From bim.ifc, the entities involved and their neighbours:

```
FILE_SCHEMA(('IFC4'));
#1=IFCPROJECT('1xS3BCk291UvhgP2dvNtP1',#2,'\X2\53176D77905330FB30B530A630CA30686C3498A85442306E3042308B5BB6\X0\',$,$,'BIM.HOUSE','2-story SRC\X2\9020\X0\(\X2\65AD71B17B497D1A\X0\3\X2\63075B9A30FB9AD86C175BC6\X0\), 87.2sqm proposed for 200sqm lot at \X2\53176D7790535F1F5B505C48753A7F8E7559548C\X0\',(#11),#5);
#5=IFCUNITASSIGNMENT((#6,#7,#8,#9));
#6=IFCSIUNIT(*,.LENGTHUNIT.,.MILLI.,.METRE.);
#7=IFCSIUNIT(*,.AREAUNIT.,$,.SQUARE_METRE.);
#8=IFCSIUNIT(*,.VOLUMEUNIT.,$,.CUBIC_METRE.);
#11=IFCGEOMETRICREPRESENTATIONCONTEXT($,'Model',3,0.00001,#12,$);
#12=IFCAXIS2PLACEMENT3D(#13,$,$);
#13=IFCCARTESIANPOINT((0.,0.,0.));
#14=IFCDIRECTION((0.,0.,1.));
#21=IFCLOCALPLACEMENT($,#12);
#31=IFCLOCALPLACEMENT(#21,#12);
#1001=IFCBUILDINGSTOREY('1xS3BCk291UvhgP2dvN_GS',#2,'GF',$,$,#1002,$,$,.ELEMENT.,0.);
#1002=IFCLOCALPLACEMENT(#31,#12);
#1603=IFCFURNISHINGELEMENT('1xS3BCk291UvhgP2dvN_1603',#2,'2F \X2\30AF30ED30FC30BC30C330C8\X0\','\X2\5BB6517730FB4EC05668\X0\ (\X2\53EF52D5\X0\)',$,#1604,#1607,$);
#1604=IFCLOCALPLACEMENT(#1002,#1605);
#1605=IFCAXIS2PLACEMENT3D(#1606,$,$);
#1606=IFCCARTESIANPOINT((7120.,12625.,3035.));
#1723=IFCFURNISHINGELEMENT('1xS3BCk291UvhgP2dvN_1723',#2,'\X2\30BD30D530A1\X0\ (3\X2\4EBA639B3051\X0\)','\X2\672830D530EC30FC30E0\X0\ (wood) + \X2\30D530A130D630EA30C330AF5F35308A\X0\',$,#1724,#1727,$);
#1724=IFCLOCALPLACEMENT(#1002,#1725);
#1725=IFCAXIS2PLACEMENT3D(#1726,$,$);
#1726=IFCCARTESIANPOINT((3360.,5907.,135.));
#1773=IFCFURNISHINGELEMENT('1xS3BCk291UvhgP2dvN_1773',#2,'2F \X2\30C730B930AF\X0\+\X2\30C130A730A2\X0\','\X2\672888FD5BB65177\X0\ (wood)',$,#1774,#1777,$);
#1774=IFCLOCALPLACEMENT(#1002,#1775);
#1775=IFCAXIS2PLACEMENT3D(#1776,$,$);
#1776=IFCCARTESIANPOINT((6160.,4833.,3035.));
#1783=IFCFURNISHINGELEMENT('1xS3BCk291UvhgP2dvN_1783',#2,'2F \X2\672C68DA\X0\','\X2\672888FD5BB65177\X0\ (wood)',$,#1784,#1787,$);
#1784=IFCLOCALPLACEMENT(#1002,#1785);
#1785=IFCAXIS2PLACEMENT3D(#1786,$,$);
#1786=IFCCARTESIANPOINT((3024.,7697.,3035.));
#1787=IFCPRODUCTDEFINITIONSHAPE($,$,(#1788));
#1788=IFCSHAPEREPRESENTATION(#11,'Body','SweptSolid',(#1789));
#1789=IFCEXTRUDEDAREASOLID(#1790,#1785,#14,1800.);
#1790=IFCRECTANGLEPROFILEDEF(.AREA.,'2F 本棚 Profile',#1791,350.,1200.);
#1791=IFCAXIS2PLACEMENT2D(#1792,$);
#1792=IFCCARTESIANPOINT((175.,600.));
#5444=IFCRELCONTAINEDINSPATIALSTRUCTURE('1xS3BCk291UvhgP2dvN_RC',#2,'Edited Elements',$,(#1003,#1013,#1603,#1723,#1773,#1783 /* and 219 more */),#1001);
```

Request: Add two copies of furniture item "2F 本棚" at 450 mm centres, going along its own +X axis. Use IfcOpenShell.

```python
import ifcopenshell
import ifcopenshell.api.geometry
import ifcopenshell.api.root
import ifcopenshell.util.element
import ifcopenshell.util.placement
import ifcopenshell.util.unit

model = ifcopenshell.open("bim.ifc")
unit_scale = ifcopenshell.util.unit.calculate_unit_scale(model)


def reuse_history(source, copy):
    """copy_class also copies each property set's owner history, people and application; keep the originals."""
    for rel in copy.IsDefinedBy:
        if rel.is_a("IfcRelDefinesByProperties") and (history := rel.RelatingPropertyDefinition.OwnerHistory):
            rel.RelatingPropertyDefinition.OwnerHistory = source.OwnerHistory
            ifcopenshell.util.element.remove_deep2(model, history)


source = model.by_id(1783)
base = ifcopenshell.util.placement.get_local_placement(source.ObjectPlacement)
step = base[:3, 0] * 0.45 / unit_scale

for i in range(1, 3):
    copy = ifcopenshell.api.root.copy_class(model, product=source)
    copy.Representation = ifcopenshell.util.element.copy_deep(
        model, source.Representation, exclude=["IfcGeometricRepresentationContext", "IfcRepresentationMap"]
    )
    reuse_history(source, copy)
    matrix = base.copy()
    matrix[:3, 3] += i * step
    print("added at", matrix[:3, 3].round(3) + 0.0)
    ifcopenshell.api.geometry.edit_object_placement(model, product=copy, matrix=matrix, is_si=False)

model.write("bim_updated.ifc")
```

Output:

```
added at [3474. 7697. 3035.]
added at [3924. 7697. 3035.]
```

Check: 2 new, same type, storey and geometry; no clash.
